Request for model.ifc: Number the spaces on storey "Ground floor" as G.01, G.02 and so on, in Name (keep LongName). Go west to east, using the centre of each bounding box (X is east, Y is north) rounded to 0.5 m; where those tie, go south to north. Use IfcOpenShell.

First a look at what the model holds.

```python
import ifcopenshell
import ifcopenshell.util.element
import ifcopenshell.util.placement

model = ifcopenshell.open("model.ifc")
print(model.schema)
storey = next(s for s in model.by_type("IfcBuildingStorey") if s.Name == "Ground floor")
spaces = [e for e in ifcopenshell.util.element.get_decomposition(storey) if e.is_a("IfcSpace")]
for e in sorted(spaces, key=lambda e: e.id()):
    origin = ifcopenshell.util.placement.get_local_placement(e.ObjectPlacement)[:3, 3]
    print(e.id(), e.Name, e.LongName, origin.round(2) + 0.0, sep=" | ")
```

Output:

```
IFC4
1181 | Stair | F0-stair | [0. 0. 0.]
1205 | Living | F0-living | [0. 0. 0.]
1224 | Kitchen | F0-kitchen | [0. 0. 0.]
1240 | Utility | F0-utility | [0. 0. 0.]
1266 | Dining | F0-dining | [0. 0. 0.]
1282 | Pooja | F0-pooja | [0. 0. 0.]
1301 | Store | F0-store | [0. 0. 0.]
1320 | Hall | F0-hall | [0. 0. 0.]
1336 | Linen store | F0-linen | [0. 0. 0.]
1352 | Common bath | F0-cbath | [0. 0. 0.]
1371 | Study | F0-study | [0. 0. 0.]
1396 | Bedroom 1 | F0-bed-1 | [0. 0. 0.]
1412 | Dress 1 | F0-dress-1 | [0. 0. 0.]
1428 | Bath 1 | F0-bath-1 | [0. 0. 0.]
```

```python
import ifcopenshell
import ifcopenshell.geom
import ifcopenshell.util.element
import ifcopenshell.util.shape

model = ifcopenshell.open("model.ifc")
settings = ifcopenshell.geom.settings()
settings.set("use-world-coords", True)


def centre(element):
    shape = ifcopenshell.geom.create_shape(settings, element)
    return ifcopenshell.util.shape.get_bbox_centroid(shape.geometry)


storey = next(s for s in model.by_type("IfcBuildingStorey") if s.Name == "Ground floor")
spaces = [e for e in ifcopenshell.util.element.get_decomposition(storey) if e.is_a("IfcSpace")]

# Insertion points can sit at a corner or the storey origin, so sort by the geometry (in metres).
centres = {e: centre(e) for e in spaces}
spaces.sort(key=lambda e: (round(centres[e][0] / 0.5), centres[e][1]))

for i, e in enumerate(spaces, start=1):
    number = f"G.{i:02d}"
    e.Name = number
    print(e.id(), number)

model.write("model_rev.ifc")
```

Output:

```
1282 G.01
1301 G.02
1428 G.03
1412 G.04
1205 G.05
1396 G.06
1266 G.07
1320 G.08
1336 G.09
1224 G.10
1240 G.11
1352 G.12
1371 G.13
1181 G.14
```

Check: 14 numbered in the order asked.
